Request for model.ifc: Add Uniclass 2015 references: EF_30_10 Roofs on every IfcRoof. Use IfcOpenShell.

First a look at what the model holds.

```python
import ifcopenshell

model = ifcopenshell.open("model.ifc")
print(model.schema)
print("classifications:", [c.Name for c in model.by_type("IfcClassification")])
for ifc_class in ("IfcDoor", "IfcRoof", "IfcStair", "IfcWall", "IfcWindow"):
    print(ifc_class, len(model.by_type(ifc_class)))
```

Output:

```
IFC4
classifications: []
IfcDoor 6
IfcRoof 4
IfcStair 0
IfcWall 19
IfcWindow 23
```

```python
import ifcopenshell
import ifcopenshell.api.classification

model = ifcopenshell.open("model.ifc")

system = ifcopenshell.api.classification.add_classification(model, classification="Uniclass 2015")

codes = {
    "IfcRoof": ("EF_30_10", "Roofs"),
}
for ifc_class, (code, name) in codes.items():
    products = model.by_type(ifc_class)
    ifcopenshell.api.classification.add_reference(
        model, products=products, classification=system, identification=code, name=name
    )
    print(code, len(products))

model.write("model_edited.ifc")
```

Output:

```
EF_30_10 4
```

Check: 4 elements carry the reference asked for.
